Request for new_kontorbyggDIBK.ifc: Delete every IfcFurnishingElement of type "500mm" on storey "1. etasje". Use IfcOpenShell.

First a look at what the model holds.

```python
import ifcopenshell
import ifcopenshell.util.element

model = ifcopenshell.open("new_kontorbyggDIBK.ifc")
print(model.schema)
storey = next(s for s in model.by_type("IfcBuildingStorey") if s.Name == "1. etasje")
furniture = [e for e in ifcopenshell.util.element.get_decomposition(storey) if e.is_a("IfcFurnishingElement")]
seen = {}
for e in furniture:
    element_type = ifcopenshell.util.element.get_type(e)
    name = element_type.Name if element_type not in (None, e) else None
    seen[name] = seen.get(name, 0) + 1
for name, count in sorted(seen.items(), key=str):
    print(count, "x", name)
```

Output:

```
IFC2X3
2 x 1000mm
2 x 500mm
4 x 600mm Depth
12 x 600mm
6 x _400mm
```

```python
import ifcopenshell
import ifcopenshell.api.root
import ifcopenshell.util.element

model = ifcopenshell.open("new_kontorbyggDIBK.ifc")

storey = next(s for s in model.by_type("IfcBuildingStorey") if s.Name == "1. etasje")
furniture = [e for e in ifcopenshell.util.element.get_decomposition(storey) if e.is_a("IfcFurnishingElement")]
targets = [e for e in furniture if (t := ifcopenshell.util.element.get_type(e)) not in (None, e) and t.Name == "500mm"]

for e in targets:
    ifcopenshell.api.root.remove_product(model, product=e)
print(len(targets), "removed")

model.write("new_kontorbyggDIBK-out.ifc")
```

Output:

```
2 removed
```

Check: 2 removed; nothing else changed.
